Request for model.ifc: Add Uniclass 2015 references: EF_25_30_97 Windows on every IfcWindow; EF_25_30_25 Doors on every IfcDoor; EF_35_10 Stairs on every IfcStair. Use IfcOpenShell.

First a look at what the model holds.

```python
import ifcopenshell

model = ifcopenshell.open("model.ifc")
print(model.schema)
print("classifications:", [c.Name for c in model.by_type("IfcClassification")])
for ifc_class in ("IfcDoor", "IfcRoof", "IfcStair", "IfcWall", "IfcWindow"):
    print(ifc_class, len(model.by_type(ifc_class)))
```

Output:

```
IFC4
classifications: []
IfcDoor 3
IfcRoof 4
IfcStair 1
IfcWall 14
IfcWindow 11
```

```python
import ifcopenshell
import ifcopenshell.api.classification

model = ifcopenshell.open("model.ifc")

system = ifcopenshell.api.classification.add_classification(model, classification="Uniclass 2015")

codes = {
    "IfcWindow": ("EF_25_30_97", "Windows"),
    "IfcDoor": ("EF_25_30_25", "Doors"),
    "IfcStair": ("EF_35_10", "Stairs"),
}
for ifc_class, (code, name) in codes.items():
    products = model.by_type(ifc_class)
    ifcopenshell.api.classification.add_reference(
        model, products=products, classification=system, identification=code, name=name
    )
    print(code, len(products))

model.write("model_edited.ifc")
```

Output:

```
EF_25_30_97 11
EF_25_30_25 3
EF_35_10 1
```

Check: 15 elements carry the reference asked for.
